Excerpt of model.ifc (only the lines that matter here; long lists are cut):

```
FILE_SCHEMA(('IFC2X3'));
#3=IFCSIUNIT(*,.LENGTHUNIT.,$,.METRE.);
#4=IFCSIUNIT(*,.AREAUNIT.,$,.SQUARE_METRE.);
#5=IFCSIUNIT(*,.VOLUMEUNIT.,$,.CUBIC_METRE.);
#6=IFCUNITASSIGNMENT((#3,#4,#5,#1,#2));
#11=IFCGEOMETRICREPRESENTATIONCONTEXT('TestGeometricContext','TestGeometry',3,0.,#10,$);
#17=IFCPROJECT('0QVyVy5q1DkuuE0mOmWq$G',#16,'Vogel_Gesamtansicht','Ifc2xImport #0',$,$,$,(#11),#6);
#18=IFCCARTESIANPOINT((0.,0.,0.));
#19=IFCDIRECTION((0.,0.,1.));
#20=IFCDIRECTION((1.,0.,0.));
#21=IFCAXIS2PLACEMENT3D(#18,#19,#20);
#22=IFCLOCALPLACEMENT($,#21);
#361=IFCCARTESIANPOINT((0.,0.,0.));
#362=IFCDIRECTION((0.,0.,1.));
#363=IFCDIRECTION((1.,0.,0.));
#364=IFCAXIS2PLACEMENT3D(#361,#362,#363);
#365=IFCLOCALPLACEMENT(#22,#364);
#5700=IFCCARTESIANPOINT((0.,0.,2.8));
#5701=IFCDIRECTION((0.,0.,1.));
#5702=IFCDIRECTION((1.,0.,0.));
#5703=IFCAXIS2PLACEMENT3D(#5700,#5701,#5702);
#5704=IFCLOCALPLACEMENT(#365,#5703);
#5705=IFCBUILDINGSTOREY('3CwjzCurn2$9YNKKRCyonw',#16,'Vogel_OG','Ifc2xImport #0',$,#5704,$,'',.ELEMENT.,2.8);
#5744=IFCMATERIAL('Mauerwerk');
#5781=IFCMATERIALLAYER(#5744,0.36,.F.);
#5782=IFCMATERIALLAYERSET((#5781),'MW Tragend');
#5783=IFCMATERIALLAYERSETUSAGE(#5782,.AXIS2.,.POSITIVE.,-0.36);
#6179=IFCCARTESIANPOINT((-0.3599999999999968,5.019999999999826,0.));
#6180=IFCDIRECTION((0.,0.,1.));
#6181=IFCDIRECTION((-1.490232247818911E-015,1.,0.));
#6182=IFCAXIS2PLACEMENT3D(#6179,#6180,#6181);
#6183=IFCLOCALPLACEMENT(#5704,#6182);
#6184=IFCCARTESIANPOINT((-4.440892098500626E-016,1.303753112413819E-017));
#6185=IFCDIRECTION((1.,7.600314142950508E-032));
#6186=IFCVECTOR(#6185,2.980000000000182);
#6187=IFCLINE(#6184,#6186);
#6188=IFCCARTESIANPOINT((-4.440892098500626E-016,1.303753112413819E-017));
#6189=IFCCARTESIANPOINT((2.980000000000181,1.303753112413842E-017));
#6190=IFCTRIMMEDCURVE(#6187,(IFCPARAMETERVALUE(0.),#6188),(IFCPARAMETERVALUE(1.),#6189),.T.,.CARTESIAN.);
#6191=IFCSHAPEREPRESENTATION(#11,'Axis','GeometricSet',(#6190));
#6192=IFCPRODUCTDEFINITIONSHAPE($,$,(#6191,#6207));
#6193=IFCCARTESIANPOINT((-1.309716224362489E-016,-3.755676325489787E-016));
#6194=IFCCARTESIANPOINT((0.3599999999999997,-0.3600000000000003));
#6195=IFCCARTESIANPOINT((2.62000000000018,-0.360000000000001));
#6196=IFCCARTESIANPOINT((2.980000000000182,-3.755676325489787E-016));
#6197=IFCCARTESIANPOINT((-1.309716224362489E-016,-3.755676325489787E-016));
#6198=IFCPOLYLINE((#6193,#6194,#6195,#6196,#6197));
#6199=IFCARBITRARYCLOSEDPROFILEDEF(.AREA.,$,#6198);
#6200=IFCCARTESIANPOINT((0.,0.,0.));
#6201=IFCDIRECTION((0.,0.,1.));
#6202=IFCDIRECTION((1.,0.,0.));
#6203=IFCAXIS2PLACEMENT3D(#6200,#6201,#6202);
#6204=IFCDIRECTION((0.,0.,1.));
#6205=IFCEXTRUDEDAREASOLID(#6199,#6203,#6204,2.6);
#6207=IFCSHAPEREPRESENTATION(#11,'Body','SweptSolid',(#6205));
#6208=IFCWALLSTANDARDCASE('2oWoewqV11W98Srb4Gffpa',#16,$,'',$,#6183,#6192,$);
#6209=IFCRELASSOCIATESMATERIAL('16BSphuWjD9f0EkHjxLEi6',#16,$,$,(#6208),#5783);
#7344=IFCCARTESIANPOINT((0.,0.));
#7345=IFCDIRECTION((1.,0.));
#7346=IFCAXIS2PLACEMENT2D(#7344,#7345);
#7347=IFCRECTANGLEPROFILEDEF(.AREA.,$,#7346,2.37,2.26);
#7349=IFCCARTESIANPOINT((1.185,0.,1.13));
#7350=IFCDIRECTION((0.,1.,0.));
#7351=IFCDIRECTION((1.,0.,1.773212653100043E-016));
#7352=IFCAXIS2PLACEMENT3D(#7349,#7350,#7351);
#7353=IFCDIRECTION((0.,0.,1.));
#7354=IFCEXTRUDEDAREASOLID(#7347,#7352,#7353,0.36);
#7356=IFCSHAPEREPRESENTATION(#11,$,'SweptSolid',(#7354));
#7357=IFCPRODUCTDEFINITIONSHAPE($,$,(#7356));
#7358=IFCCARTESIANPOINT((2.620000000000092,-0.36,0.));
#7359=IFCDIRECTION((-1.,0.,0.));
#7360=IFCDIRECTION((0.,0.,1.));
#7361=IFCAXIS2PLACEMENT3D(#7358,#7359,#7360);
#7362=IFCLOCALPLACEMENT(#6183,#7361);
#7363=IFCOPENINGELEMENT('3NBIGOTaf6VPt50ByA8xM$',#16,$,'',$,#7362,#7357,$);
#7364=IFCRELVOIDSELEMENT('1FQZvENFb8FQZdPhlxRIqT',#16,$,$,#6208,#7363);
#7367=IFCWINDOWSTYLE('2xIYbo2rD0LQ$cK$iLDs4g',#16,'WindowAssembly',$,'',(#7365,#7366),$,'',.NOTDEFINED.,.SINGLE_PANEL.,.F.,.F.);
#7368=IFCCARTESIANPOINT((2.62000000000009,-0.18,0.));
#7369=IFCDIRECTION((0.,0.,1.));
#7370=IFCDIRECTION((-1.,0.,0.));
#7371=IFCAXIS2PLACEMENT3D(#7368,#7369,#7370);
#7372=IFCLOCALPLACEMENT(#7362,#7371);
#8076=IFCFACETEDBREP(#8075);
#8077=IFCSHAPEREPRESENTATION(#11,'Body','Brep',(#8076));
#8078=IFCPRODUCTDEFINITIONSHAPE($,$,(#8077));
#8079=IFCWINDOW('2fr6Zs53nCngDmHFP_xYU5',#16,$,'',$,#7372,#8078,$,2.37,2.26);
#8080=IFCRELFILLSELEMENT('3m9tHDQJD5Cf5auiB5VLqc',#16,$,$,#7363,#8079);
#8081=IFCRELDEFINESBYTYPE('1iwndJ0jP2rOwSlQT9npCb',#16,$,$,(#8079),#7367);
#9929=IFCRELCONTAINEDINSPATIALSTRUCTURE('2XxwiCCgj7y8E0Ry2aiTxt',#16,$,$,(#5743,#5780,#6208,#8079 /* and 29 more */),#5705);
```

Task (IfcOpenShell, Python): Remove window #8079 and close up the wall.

```python
import ifcopenshell
import ifcopenshell.api.feature
import ifcopenshell.api.root
import ifcopenshell.geom
import ifcopenshell.util.shape

model = ifcopenshell.open("model.ifc")
settings = ifcopenshell.geom.settings()


def volume(element):
    """Net volume in cubic metres, openings subtracted."""
    shape = ifcopenshell.geom.create_shape(settings, element)
    return ifcopenshell.util.shape.get_volume(shape.geometry)


window = model.by_id(8079)
opening = window.FillsVoids[0].RelatingOpeningElement
wall = opening.VoidsElements[0].RelatingBuildingElement
before = volume(wall)

ifcopenshell.api.root.remove_product(model, product=window)
ifcopenshell.api.feature.remove_feature(model, feature=opening)

after = volume(wall)

print(f"wall volume {before:.3f} -> {after:.3f} m3")

model.write("model_v2.ifc")
```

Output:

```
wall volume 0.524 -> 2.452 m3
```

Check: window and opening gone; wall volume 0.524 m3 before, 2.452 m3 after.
